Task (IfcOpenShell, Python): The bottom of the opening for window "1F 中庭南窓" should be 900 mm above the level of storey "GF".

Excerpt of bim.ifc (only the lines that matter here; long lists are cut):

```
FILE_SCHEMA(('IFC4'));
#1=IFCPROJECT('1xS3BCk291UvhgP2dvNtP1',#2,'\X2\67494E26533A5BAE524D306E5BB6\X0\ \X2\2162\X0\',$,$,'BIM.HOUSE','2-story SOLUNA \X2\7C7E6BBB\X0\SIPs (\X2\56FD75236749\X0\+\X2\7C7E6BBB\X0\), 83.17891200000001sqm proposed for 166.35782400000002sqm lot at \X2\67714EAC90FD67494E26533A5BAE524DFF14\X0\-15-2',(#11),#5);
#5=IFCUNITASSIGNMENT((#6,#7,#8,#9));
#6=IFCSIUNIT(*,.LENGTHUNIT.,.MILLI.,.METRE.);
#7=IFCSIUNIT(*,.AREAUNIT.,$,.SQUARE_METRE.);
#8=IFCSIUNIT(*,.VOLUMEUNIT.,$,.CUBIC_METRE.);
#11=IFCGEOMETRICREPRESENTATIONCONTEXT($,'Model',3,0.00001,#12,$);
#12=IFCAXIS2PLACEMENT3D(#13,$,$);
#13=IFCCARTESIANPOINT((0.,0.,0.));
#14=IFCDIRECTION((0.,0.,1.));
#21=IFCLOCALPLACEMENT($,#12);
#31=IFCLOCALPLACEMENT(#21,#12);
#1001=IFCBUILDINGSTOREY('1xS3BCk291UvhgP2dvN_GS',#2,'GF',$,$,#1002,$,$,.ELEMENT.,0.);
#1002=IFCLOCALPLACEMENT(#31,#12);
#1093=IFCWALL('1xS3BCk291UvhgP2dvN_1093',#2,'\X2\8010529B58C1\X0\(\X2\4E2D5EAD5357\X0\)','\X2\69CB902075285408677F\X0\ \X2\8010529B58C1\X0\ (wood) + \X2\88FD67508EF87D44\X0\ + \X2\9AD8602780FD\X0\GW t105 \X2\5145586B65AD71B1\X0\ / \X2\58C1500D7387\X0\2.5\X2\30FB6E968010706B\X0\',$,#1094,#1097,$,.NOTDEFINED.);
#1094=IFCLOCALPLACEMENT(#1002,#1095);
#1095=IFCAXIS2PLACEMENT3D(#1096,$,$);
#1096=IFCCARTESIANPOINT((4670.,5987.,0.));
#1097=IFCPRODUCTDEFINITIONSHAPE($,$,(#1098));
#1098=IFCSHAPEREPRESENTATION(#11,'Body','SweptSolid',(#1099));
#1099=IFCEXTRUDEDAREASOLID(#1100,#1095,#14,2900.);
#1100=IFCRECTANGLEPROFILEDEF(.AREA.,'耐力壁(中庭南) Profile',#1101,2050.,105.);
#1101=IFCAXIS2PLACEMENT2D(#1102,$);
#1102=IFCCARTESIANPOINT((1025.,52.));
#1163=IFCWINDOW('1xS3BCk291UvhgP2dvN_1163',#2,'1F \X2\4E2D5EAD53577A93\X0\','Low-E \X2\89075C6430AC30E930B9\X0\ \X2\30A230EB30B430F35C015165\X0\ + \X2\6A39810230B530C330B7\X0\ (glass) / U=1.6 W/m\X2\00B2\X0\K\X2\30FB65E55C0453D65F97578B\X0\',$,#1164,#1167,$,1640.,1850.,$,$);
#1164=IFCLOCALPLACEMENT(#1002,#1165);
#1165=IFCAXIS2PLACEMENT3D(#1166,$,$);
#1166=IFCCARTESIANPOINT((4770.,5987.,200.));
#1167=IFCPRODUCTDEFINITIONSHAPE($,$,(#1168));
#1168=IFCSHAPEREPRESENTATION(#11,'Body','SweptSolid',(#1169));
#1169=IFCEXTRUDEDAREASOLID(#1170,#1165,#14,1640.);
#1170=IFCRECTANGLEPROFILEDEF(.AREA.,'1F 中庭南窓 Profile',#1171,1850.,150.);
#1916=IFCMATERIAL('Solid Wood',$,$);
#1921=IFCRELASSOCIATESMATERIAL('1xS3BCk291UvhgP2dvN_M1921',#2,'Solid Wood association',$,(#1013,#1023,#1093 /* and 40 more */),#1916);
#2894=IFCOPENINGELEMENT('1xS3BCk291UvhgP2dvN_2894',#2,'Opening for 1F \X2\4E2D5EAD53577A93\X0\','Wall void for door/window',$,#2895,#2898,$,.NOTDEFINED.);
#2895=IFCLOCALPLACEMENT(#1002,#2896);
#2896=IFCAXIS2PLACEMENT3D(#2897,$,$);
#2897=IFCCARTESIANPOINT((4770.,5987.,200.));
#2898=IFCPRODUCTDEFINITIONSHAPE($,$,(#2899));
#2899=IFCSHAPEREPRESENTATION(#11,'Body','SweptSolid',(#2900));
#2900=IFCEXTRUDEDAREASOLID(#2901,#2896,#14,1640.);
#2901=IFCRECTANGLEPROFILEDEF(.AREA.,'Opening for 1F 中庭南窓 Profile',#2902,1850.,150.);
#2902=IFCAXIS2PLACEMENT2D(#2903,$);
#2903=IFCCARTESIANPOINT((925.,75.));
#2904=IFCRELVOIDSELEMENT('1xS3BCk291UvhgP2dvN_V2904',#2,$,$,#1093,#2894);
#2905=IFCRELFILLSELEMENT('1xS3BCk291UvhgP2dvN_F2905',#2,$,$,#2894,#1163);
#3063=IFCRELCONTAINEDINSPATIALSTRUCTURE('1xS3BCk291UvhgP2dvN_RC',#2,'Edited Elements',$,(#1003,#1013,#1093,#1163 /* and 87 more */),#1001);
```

```python
import numpy as np
import ifcopenshell
import ifcopenshell.api.geometry
import ifcopenshell.geom
import ifcopenshell.util.element
import ifcopenshell.util.placement
import ifcopenshell.util.shape
import ifcopenshell.util.unit

model = ifcopenshell.open("bim.ifc")
unit_scale = ifcopenshell.util.unit.calculate_unit_scale(model)

window = model.by_id(1163)
opening = window.FillsVoids[0].RelatingOpeningElement
storey = ifcopenshell.util.element.get_container(window, ifc_class="IfcBuildingStorey")
level = ifcopenshell.util.placement.get_local_placement(storey.ObjectPlacement)[2, 3]

# The opening's origin need not be at the sill, so measure its lowest point.
shape = ifcopenshell.geom.create_shape(ifcopenshell.geom.settings(), opening)
bottom = ifcopenshell.util.shape.get_shape_bottom_elevation(shape, shape.geometry) / unit_scale
dz = level + 0.9 / unit_scale - bottom

shift = np.array([0.0, 0.0, dz])
# The window is not placed relative to its opening, so move both.
for product in (opening, window):
    matrix = ifcopenshell.util.placement.get_local_placement(product.ObjectPlacement)
    matrix[:3, 3] += shift
    ifcopenshell.api.geometry.edit_object_placement(model, product=product, matrix=matrix, is_si=False)

print(f"moved by {dz * unit_scale:+.3f} m")

model.write("bim_updated.ifc")
```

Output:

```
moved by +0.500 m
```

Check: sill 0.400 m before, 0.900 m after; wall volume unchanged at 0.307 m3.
